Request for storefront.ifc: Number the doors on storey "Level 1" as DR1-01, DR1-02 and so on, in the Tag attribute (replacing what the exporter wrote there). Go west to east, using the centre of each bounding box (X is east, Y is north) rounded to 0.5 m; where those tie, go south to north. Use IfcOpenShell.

First a look at what the model holds.

```python
import ifcopenshell
import ifcopenshell.util.element
import ifcopenshell.util.placement

model = ifcopenshell.open("storefront.ifc")
print(model.schema)
storey = next(s for s in model.by_type("IfcBuildingStorey") if s.Name == "Level 1")
doors = [e for e in ifcopenshell.util.element.get_decomposition(storey) if e.is_a("IfcDoor")]
for e in sorted(doors, key=lambda e: e.id()):
    origin = ifcopenshell.util.placement.get_local_placement(e.ObjectPlacement)[:3, 3]
    print(e.id(), e.Tag, e.Name, origin.round(2) + 0.0, sep=" | ")
```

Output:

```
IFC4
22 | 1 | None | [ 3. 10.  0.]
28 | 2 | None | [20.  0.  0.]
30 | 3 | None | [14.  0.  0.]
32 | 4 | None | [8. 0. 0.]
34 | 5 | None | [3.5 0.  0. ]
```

```python
import ifcopenshell
import ifcopenshell.geom
import ifcopenshell.util.element
import ifcopenshell.util.shape

model = ifcopenshell.open("storefront.ifc")
settings = ifcopenshell.geom.settings()
settings.set("use-world-coords", True)


def centre(element):
    shape = ifcopenshell.geom.create_shape(settings, element)
    return ifcopenshell.util.shape.get_bbox_centroid(shape.geometry)


storey = next(s for s in model.by_type("IfcBuildingStorey") if s.Name == "Level 1")
doors = [e for e in ifcopenshell.util.element.get_decomposition(storey) if e.is_a("IfcDoor")]

# Insertion points can sit at a corner or the storey origin, so sort by the geometry (in metres).
centres = {e: centre(e) for e in doors}
doors.sort(key=lambda e: (round(centres[e][0] / 0.5), centres[e][1]))

for i, e in enumerate(doors, start=1):
    number = f"DR1-{i:02d}"
    e.Tag = number
    print(e.id(), number)

model.write("storefront_edited.ifc")
```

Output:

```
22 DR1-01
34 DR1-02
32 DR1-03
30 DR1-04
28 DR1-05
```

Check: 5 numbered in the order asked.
